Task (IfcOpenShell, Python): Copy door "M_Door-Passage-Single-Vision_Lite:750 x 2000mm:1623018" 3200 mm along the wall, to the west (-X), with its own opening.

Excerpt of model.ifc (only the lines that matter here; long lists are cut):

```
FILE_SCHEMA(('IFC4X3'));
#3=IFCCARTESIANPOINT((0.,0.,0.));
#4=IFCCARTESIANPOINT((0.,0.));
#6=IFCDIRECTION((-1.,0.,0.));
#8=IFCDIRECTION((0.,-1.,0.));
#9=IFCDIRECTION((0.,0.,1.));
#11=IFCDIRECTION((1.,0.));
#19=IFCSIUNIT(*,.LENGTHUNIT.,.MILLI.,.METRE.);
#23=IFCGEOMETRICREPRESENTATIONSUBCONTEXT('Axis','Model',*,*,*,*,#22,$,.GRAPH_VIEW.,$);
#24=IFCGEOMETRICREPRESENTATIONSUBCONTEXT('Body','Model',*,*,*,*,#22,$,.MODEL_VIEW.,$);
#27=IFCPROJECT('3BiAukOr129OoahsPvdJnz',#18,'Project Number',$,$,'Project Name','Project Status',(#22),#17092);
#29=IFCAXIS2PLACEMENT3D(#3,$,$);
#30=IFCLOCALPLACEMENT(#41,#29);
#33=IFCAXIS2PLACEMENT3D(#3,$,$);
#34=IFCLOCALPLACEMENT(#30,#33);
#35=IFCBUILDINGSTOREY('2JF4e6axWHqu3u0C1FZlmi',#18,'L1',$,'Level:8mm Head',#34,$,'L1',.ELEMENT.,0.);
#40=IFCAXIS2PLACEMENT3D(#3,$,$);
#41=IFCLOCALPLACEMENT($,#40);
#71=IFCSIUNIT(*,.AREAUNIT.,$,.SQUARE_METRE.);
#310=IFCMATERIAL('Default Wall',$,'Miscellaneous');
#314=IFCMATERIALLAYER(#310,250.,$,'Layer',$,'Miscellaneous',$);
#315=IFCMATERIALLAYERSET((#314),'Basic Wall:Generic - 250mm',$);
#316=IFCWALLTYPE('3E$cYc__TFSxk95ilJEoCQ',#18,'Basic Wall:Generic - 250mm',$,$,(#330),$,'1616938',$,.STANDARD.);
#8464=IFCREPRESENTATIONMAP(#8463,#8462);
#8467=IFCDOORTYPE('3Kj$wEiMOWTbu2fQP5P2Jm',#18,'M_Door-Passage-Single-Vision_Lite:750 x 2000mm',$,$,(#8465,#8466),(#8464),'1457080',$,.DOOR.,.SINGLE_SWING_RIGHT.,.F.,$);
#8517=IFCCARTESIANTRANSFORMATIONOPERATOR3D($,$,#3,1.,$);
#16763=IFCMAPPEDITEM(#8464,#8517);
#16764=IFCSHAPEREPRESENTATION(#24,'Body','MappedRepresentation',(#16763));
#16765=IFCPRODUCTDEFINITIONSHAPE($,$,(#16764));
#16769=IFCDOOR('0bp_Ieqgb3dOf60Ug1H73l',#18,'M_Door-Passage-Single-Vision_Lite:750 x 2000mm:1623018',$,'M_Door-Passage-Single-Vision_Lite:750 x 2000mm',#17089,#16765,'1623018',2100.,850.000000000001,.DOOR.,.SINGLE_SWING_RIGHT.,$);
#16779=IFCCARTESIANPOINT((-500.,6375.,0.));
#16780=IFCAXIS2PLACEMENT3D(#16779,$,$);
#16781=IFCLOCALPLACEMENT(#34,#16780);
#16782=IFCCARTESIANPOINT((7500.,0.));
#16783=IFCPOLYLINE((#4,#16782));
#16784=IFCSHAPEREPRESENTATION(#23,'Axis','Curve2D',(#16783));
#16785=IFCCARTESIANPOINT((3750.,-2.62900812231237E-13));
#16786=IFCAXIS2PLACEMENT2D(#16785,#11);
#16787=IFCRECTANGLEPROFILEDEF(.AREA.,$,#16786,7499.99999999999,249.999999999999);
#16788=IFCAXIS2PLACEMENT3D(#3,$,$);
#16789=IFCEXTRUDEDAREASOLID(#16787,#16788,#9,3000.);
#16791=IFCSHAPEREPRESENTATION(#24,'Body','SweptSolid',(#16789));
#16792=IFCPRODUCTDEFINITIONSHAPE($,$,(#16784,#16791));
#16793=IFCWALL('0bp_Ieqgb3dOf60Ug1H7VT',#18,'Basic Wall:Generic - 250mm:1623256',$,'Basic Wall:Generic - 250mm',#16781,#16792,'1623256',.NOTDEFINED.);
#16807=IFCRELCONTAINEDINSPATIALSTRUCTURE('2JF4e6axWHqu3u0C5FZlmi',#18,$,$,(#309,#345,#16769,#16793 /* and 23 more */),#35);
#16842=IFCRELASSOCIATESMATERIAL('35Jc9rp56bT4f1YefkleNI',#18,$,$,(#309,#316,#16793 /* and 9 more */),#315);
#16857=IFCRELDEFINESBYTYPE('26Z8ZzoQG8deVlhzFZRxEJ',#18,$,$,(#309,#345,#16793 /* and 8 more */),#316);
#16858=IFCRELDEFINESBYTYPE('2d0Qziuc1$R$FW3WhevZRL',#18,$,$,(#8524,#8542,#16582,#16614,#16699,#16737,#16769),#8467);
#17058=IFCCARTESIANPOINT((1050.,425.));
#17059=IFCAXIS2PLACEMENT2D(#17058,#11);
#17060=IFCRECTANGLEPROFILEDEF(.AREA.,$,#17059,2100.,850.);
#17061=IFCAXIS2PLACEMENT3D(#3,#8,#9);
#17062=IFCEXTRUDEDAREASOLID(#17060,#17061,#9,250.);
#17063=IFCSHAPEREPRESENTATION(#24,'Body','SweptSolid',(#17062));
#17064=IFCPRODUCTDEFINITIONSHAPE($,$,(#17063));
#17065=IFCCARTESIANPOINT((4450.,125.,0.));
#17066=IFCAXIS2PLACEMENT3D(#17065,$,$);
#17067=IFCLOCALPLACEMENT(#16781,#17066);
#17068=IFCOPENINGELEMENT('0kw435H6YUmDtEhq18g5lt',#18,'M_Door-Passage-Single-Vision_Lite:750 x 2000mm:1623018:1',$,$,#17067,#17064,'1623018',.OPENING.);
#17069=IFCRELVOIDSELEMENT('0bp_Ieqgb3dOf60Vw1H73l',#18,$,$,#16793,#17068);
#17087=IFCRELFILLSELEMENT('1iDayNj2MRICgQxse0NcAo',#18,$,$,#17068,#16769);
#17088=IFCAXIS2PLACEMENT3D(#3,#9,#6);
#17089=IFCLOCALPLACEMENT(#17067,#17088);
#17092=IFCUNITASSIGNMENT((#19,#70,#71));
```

```python
import ifcopenshell
import ifcopenshell.api.feature
import ifcopenshell.api.geometry
import ifcopenshell.api.root
import ifcopenshell.geom
import ifcopenshell.util.element
import ifcopenshell.util.placement
import ifcopenshell.util.shape
import ifcopenshell.util.unit

model = ifcopenshell.open("model.ifc")
unit_scale = ifcopenshell.util.unit.calculate_unit_scale(model)
settings = ifcopenshell.geom.settings()


def volume(element):
    """Net volume in cubic metres, openings subtracted."""
    shape = ifcopenshell.geom.create_shape(settings, element)
    return ifcopenshell.util.shape.get_volume(shape.geometry)


def reuse_history(source, copy):
    """copy_class also copies each property set's owner history, people and application; keep the originals."""
    for rel in copy.IsDefinedBy:
        if rel.is_a("IfcRelDefinesByProperties") and (history := rel.RelatingPropertyDefinition.OwnerHistory):
            rel.RelatingPropertyDefinition.OwnerHistory = source.OwnerHistory
            ifcopenshell.util.element.remove_deep2(model, history)


door = model.by_guid("0bp_Ieqgb3dOf60Ug1H73l")
opening = door.FillsVoids[0].RelatingOpeningElement
wall = opening.VoidsElements[0].RelatingBuildingElement
before = volume(wall)
shift = ifcopenshell.util.placement.get_local_placement(wall.ObjectPlacement)[:3, 0] * -3.2 / unit_scale

# copy_class copies the void relationship, type, container and properties, but no geometry.
new_opening = ifcopenshell.api.root.copy_class(model, product=opening)
new_opening.Representation = ifcopenshell.util.element.copy_deep(
    model, opening.Representation, exclude=["IfcGeometricRepresentationContext", "IfcRepresentationMap"]
)
new_opening.Name = "M_Door-Passage-Single-Vision_Lite:750 x 2000mm"
new_opening.Tag = None
new_door = ifcopenshell.api.root.copy_class(model, product=door)
new_door.Representation = ifcopenshell.util.element.copy_deep(
    model, door.Representation, exclude=["IfcGeometricRepresentationContext", "IfcRepresentationMap"]
)
new_door.Name = "M_Door-Passage-Single-Vision_Lite:750 x 2000mm"
new_door.Tag = None
reuse_history(door, new_door)
ifcopenshell.api.feature.add_filling(model, opening=new_opening, element=new_door)

for old, new in ((opening, new_opening), (door, new_door)):
    matrix = ifcopenshell.util.placement.get_local_placement(old.ObjectPlacement)
    matrix[:3, 3] += shift
    ifcopenshell.api.geometry.edit_object_placement(model, product=new, matrix=matrix, is_si=False)

after = volume(wall)

print(f"wall volume {before:.3f} -> {after:.3f} m3")

model.write("model_updated.ifc")
```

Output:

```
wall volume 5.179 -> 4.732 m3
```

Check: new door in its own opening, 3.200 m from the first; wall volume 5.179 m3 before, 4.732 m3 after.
